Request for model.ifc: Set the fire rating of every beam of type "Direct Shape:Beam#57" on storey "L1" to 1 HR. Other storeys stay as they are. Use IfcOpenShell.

First a look at what the model holds.

```python
import ifcopenshell
import ifcopenshell.util.element

model = ifcopenshell.open("model.ifc")
print(model.schema)
storey = next(s for s in model.by_type("IfcBuildingStorey") if s.Name == "L1")
beams = [e for e in ifcopenshell.util.element.get_decomposition(storey) if e.is_a("IfcBeam")]
seen = {}
for e in beams:
    element_type = ifcopenshell.util.element.get_type(e)
    key = (element_type.Name if element_type != e and element_type else None, ifcopenshell.util.element.get_pset(e, "Pset_BeamCommon", "FireRating"))
    seen[key] = seen.get(key, 0) + 1
for (name, value), count in sorted(seen.items(), key=str):
    print(count, "x", name, "|", value)
```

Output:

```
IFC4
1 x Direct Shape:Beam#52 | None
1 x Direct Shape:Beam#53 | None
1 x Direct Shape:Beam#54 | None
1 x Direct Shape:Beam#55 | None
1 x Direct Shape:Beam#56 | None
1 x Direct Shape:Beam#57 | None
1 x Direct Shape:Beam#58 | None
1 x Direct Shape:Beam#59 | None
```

```python
import ifcopenshell
import ifcopenshell.api.pset
import ifcopenshell.util.element

model = ifcopenshell.open("model.ifc")

storey = next(s for s in model.by_type("IfcBuildingStorey") if s.Name == "L1")
beams = [e for e in ifcopenshell.util.element.get_decomposition(storey) if e.is_a("IfcBeam")]

count = 0
for e in beams:
    element_type = ifcopenshell.util.element.get_type(e)
    if element_type in (None, e) or element_type.Name != "Direct Shape:Beam#57":
        continue
    # add_pset returns the element's existing set when there is one.
    pset = ifcopenshell.api.pset.add_pset(model, product=e, name="Pset_BeamCommon")
    ifcopenshell.api.pset.edit_pset(model, pset=pset, properties={"FireRating": "1 HR"})
    count += 1

print(count, "beams updated")

model.write("model-out.ifc")
```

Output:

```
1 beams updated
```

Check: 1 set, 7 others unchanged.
